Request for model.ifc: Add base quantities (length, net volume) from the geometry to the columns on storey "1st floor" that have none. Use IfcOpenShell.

First a look at what the model holds.

```python
import ifcopenshell
import ifcopenshell.util.element
import ifcopenshell.util.unit

model = ifcopenshell.open("model.ifc")
print(model.schema)
for unit_type in ("LENGTHUNIT", "AREAUNIT", "VOLUMEUNIT"):
    print(unit_type, ifcopenshell.util.unit.calculate_unit_scale(model, unit_type))
storey = next(s for s in model.by_type("IfcBuildingStorey") if s.Name == "1st floor")
columns = [e for e in ifcopenshell.util.element.get_decomposition(storey) if e.is_a("IfcColumn")]
for e in sorted(columns, key=lambda e: e.id()):
    print(e.id(), e.is_a(), e.Name, list(ifcopenshell.util.element.get_psets(e, qtos_only=True)), sep=" | ")
```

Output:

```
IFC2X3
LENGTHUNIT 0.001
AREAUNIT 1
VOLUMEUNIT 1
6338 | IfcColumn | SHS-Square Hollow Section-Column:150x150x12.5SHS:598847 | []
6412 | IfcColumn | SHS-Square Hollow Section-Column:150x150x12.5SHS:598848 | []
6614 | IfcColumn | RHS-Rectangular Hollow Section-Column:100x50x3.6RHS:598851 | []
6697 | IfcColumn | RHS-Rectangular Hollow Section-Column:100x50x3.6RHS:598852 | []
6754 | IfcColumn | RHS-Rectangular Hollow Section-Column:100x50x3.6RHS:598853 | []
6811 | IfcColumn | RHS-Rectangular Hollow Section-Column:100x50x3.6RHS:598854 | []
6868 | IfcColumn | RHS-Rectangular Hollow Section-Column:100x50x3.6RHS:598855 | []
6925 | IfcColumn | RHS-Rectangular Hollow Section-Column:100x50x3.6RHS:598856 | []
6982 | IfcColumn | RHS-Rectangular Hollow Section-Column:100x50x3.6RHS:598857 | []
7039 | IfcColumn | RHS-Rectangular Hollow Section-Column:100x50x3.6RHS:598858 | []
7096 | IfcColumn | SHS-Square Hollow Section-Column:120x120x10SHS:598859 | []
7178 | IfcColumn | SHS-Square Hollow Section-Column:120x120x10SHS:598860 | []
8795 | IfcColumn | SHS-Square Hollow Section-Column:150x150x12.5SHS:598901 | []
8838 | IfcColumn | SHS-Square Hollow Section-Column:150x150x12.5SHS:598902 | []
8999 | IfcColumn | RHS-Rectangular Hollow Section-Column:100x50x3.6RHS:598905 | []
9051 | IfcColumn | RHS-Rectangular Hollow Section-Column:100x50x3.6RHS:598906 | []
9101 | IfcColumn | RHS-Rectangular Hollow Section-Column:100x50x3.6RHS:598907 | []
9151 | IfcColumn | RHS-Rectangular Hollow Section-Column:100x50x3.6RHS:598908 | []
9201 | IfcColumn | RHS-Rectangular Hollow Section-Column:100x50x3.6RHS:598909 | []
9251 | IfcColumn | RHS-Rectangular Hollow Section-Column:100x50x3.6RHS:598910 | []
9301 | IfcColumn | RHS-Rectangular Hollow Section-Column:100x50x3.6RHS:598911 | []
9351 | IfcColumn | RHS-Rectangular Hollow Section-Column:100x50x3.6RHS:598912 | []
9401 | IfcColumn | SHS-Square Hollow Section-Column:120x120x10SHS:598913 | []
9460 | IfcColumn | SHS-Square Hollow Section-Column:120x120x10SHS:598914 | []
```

```python
import ifcopenshell
import ifcopenshell.api.pset
import ifcopenshell.geom
import ifcopenshell.util.element
import ifcopenshell.util.shape
import ifcopenshell.util.unit

model = ifcopenshell.open("model.ifc")
unit_scale = ifcopenshell.util.unit.calculate_unit_scale(model)
volume_scale = ifcopenshell.util.unit.calculate_unit_scale(model, "VOLUMEUNIT")
settings = ifcopenshell.geom.settings()

storey = next(s for s in model.by_type("IfcBuildingStorey") if s.Name == "1st floor")
columns = [e for e in ifcopenshell.util.element.get_decomposition(storey) if e.is_a("IfcColumn")]

for e in sorted(columns, key=lambda e: e.id()):
    if ifcopenshell.util.element.get_psets(e, qtos_only=True, should_inherit=False):
        continue
    # Geometry comes back in metres, in the element's own axes.
    shape = ifcopenshell.geom.create_shape(settings, e)
    values = {
        "Length": ifcopenshell.util.shape.get_z(shape.geometry) / unit_scale,
        "NetVolume": ifcopenshell.util.shape.get_volume(shape.geometry) / volume_scale,
    }
    qto = ifcopenshell.api.pset.add_qto(model, product=e, name="BaseQuantities")
    ifcopenshell.api.pset.edit_qto(model, qto=qto, properties=values)
    print(e.id(), {k: round(v, 3) for k, v in values.items()})

model.write("model_rev.ifc")
```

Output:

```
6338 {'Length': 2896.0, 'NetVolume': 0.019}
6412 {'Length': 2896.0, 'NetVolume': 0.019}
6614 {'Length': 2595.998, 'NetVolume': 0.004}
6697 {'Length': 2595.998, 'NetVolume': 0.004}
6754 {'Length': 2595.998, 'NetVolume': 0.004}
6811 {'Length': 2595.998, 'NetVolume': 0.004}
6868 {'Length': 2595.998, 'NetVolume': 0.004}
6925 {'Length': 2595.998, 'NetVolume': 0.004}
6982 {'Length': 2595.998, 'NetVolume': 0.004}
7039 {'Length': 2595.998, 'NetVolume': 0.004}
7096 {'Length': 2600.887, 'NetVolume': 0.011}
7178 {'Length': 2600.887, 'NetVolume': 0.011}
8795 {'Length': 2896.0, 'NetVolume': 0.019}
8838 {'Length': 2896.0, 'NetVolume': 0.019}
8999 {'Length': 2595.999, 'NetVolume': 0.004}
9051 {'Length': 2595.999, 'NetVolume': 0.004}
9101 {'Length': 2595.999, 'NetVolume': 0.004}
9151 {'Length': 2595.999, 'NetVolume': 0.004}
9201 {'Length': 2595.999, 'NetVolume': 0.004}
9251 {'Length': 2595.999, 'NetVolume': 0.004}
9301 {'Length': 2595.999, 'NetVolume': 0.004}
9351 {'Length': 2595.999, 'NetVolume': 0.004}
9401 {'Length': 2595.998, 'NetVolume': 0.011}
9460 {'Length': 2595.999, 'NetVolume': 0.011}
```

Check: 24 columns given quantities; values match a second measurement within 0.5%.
